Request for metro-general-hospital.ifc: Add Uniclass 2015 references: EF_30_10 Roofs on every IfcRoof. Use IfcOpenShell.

First a look at what the model holds.

```python
import ifcopenshell

model = ifcopenshell.open("metro-general-hospital.ifc")
print(model.schema)
print("classifications:", [c.Name for c in model.by_type("IfcClassification")])
for ifc_class in ("IfcDoor", "IfcRoof", "IfcStair", "IfcWall", "IfcWindow"):
    print(ifc_class, len(model.by_type(ifc_class)))
```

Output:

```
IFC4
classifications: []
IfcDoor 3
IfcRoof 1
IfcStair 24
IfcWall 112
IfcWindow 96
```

```python
import ifcopenshell
import ifcopenshell.api.classification

model = ifcopenshell.open("metro-general-hospital.ifc")

system = ifcopenshell.api.classification.add_classification(model, classification="Uniclass 2015")

codes = {
    "IfcRoof": ("EF_30_10", "Roofs"),
}
for ifc_class, (code, name) in codes.items():
    products = model.by_type(ifc_class)
    ifcopenshell.api.classification.add_reference(
        model, products=products, classification=system, identification=code, name=name
    )
    print(code, len(products))

model.write("metro-general-hospital-out.ifc")
```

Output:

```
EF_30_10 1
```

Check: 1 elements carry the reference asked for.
